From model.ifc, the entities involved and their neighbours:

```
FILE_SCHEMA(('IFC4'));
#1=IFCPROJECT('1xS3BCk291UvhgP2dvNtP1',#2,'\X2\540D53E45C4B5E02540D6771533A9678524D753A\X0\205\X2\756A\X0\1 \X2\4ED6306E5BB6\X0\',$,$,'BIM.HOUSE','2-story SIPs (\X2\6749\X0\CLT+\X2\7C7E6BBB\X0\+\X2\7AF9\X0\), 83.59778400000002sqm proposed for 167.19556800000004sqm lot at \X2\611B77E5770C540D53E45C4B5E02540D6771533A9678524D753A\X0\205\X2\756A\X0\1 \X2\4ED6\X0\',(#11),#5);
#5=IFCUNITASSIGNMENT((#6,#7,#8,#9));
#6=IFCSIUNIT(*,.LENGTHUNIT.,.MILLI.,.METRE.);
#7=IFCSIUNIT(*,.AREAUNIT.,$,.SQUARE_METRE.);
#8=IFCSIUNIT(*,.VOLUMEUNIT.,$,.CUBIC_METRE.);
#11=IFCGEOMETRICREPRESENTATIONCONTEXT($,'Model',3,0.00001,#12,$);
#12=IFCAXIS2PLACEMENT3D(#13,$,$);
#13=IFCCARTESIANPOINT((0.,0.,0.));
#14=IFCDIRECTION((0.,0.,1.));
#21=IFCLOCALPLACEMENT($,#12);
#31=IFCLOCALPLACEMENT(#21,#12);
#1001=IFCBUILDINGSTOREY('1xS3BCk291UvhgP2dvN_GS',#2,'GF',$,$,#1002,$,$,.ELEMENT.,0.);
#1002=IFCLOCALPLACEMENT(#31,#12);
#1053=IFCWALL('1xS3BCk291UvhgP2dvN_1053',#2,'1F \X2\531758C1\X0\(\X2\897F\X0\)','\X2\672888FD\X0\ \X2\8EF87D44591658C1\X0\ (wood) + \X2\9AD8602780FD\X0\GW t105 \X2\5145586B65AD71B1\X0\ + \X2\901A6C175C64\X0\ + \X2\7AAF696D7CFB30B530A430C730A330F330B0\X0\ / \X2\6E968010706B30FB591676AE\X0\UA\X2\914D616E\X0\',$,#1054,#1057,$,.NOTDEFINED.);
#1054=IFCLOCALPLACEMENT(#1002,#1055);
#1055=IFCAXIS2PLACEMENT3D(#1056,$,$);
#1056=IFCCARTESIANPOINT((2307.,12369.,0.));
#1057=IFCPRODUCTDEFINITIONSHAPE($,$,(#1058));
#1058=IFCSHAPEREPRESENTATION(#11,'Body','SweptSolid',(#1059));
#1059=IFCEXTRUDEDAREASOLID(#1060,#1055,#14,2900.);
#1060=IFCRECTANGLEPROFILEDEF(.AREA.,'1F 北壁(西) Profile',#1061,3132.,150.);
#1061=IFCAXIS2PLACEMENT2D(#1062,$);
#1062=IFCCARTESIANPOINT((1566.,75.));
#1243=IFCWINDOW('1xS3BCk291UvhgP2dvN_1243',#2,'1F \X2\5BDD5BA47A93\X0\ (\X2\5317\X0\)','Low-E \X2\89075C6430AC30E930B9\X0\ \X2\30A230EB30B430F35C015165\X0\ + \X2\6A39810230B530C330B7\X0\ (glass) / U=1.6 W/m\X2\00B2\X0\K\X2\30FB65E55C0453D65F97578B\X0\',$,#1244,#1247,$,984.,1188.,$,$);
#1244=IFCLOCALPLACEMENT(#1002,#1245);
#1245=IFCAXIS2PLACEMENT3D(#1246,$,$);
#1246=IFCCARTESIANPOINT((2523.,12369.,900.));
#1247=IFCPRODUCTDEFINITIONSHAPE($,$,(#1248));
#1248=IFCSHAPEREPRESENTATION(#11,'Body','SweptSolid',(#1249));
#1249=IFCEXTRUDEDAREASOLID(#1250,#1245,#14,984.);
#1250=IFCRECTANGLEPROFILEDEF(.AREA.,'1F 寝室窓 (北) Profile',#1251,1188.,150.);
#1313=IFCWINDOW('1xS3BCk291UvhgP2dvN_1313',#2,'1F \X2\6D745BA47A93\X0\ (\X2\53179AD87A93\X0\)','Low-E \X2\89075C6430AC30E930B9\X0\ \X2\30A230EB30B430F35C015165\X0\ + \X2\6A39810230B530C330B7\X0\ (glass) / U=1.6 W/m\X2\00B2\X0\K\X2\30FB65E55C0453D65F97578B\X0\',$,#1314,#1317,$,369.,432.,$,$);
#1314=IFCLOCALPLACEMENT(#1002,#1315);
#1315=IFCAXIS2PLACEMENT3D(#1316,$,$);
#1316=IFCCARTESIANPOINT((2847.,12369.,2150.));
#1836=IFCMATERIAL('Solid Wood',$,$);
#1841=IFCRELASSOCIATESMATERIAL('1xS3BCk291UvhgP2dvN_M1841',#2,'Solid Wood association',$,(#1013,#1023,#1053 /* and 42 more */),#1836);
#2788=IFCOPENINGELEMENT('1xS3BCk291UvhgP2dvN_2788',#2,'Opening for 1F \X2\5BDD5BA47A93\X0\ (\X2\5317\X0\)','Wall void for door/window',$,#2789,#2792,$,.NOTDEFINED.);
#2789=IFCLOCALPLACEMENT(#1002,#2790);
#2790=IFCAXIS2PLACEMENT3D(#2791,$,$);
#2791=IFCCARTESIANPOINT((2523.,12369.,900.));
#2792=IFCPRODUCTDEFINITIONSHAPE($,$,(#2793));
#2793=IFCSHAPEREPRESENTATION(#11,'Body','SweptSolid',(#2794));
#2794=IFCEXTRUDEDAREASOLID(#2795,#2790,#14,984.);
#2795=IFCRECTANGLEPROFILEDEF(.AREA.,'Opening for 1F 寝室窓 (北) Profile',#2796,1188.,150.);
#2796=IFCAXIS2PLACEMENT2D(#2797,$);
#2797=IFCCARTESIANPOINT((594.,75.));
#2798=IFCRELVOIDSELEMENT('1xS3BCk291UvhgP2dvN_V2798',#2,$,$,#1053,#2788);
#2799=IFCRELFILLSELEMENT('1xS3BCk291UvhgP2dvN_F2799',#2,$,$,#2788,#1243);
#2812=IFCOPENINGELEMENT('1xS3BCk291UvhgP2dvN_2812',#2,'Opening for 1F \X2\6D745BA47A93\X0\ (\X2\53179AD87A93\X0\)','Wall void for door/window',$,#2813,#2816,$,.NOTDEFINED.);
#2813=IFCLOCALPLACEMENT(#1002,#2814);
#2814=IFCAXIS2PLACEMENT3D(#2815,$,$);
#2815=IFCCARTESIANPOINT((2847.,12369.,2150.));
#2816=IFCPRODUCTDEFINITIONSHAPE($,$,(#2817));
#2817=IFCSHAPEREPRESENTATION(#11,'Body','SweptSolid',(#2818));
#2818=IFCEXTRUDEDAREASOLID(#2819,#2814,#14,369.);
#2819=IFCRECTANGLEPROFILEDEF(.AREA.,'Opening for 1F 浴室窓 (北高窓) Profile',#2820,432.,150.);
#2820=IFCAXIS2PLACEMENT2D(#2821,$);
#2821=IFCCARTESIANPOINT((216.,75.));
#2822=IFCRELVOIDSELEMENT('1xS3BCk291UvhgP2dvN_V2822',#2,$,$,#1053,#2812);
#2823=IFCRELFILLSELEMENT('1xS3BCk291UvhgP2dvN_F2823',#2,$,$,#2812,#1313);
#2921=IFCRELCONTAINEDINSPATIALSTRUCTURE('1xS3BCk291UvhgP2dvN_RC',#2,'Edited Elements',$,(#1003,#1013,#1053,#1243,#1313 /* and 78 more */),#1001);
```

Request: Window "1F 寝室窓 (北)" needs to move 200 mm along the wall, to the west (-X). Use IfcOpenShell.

```python
import ifcopenshell
import ifcopenshell.api.geometry
import ifcopenshell.util.placement

model = ifcopenshell.open("model.ifc")

window = model.by_guid("1xS3BCk291UvhgP2dvN_1243")
opening = window.FillsVoids[0].RelatingOpeningElement
wall = opening.VoidsElements[0].RelatingBuildingElement

wall_matrix = ifcopenshell.util.placement.get_local_placement(wall.ObjectPlacement)
shift = wall_matrix[:3, 0] * -200.0
before = ifcopenshell.util.placement.get_local_placement(window.ObjectPlacement)[:3, 3].copy()

# The window is not placed relative to its opening, so move both.
for product in (opening, window):
    matrix = ifcopenshell.util.placement.get_local_placement(product.ObjectPlacement)
    matrix[:3, 3] += shift
    ifcopenshell.api.geometry.edit_object_placement(model, product=product, matrix=matrix, is_si=False)

after = ifcopenshell.util.placement.get_local_placement(window.ObjectPlacement)[:3, 3]
print("window moved by", (after - before).round(3) + 0.0)

model.write("model_v2.ifc")
```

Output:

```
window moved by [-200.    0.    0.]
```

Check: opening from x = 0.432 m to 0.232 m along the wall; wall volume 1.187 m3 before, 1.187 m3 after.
